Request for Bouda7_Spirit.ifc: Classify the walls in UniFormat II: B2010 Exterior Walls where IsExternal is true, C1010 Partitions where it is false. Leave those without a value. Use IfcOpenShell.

First a look at what the model holds.

```python
import ifcopenshell
import ifcopenshell.util.element

model = ifcopenshell.open("Bouda7_Spirit.ifc")
print(model.schema)
print("classifications:", [c.Name for c in model.by_type("IfcClassification")])
values = [ifcopenshell.util.element.get_pset(e, "Pset_WallCommon", "IsExternal") for e in model.by_type("IfcWall")]
for value in (True, False, None):
    print("IsExternal", value, values.count(value))
```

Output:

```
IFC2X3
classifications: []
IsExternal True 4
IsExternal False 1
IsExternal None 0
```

```python
import ifcopenshell
import ifcopenshell.api.classification
import ifcopenshell.util.element

model = ifcopenshell.open("Bouda7_Spirit.ifc")

# IFC2X3 requires Source and Edition and has no link from the project to the system.
system = model.create_entity("IfcClassification", Source="ASTM", Edition="E1557", Name="UniFormat II")

walls = model.by_type("IfcWall")
external = {e: ifcopenshell.util.element.get_pset(e, "Pset_WallCommon", "IsExternal") for e in walls}
for flag, code, name in ((True, "B2010", "Exterior Walls"), (False, "C1010", "Partitions")):
    products = [e for e in walls if external[e] is flag]
    ifcopenshell.api.classification.add_reference(
        model, products=products, classification=system, identification=code, name=name
    )
    print(code, len(products))

model.write("Bouda7_Spirit_edited.ifc")
```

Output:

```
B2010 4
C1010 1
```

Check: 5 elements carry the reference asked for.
